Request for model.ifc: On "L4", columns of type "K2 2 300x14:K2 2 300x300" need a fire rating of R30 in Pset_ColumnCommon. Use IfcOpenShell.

First a look at what the model holds.

```python
import ifcopenshell
import ifcopenshell.util.element

model = ifcopenshell.open("model.ifc")
print(model.schema)
storey = next(s for s in model.by_type("IfcBuildingStorey") if s.Name == "L4")
columns = [e for e in ifcopenshell.util.element.get_decomposition(storey) if e.is_a("IfcColumn")]
seen = {}
for e in columns:
    element_type = ifcopenshell.util.element.get_type(e)
    key = (element_type.Name if element_type != e and element_type else None, ifcopenshell.util.element.get_pset(e, "Pset_ColumnCommon", "FireRating"))
    seen[key] = seen.get(key, 0) + 1
for (name, value), count in sorted(seen.items(), key=str):
    print(count, "x", name, "|", value)
```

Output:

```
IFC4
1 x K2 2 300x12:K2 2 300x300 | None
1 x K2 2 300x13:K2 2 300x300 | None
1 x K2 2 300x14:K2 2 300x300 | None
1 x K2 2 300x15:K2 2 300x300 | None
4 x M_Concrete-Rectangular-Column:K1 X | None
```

```python
import ifcopenshell
import ifcopenshell.api.pset
import ifcopenshell.util.element

model = ifcopenshell.open("model.ifc")

storey = next(s for s in model.by_type("IfcBuildingStorey") if s.Name == "L4")
columns = [e for e in ifcopenshell.util.element.get_decomposition(storey) if e.is_a("IfcColumn")]

count = 0
for e in columns:
    element_type = ifcopenshell.util.element.get_type(e)
    if element_type in (None, e) or element_type.Name != "K2 2 300x14:K2 2 300x300":
        continue
    # add_pset returns the element's existing set when there is one.
    pset = ifcopenshell.api.pset.add_pset(model, product=e, name="Pset_ColumnCommon")
    ifcopenshell.api.pset.edit_pset(model, pset=pset, properties={"FireRating": "R30"})
    count += 1

print(count, "columns updated")

model.write("model_updated.ifc")
```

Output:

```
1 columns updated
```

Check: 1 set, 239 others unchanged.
